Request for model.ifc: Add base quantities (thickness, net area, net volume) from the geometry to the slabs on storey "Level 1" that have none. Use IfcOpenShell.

First a look at what the model holds.

```python
import ifcopenshell
import ifcopenshell.util.element
import ifcopenshell.util.unit

model = ifcopenshell.open("model.ifc")
print(model.schema)
for unit_type in ("LENGTHUNIT", "AREAUNIT", "VOLUMEUNIT"):
    print(unit_type, ifcopenshell.util.unit.calculate_unit_scale(model, unit_type))
storey = next(s for s in model.by_type("IfcBuildingStorey") if s.Name == "Level 1")
slabs = [e for e in ifcopenshell.util.element.get_decomposition(storey) if e.is_a("IfcSlab")]
for e in sorted(slabs, key=lambda e: e.id()):
    print(e.id(), e.is_a(), e.Name, list(ifcopenshell.util.element.get_psets(e, qtos_only=True)), sep=" | ")
```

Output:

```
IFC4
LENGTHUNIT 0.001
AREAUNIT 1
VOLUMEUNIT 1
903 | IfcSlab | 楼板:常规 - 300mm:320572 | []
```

```python
import ifcopenshell
import ifcopenshell.api.pset
import ifcopenshell.geom
import ifcopenshell.util.element
import ifcopenshell.util.shape
import ifcopenshell.util.unit

model = ifcopenshell.open("model.ifc")
unit_scale = ifcopenshell.util.unit.calculate_unit_scale(model)
area_scale = ifcopenshell.util.unit.calculate_unit_scale(model, "AREAUNIT")
volume_scale = ifcopenshell.util.unit.calculate_unit_scale(model, "VOLUMEUNIT")
settings = ifcopenshell.geom.settings()

storey = next(s for s in model.by_type("IfcBuildingStorey") if s.Name == "Level 1")
slabs = [e for e in ifcopenshell.util.element.get_decomposition(storey) if e.is_a("IfcSlab")]

for e in sorted(slabs, key=lambda e: e.id()):
    if ifcopenshell.util.element.get_psets(e, qtos_only=True, should_inherit=False):
        continue
    # Geometry comes back in metres, in the element's own axes.
    shape = ifcopenshell.geom.create_shape(settings, e)
    values = {
        "Width": ifcopenshell.util.shape.get_z(shape.geometry) / unit_scale,
        "NetArea": ifcopenshell.util.shape.get_footprint_area(shape.geometry) / area_scale,
        "NetVolume": ifcopenshell.util.shape.get_volume(shape.geometry) / volume_scale,
    }
    qto = ifcopenshell.api.pset.add_qto(model, product=e, name="Qto_SlabBaseQuantities")
    ifcopenshell.api.pset.edit_qto(model, qto=qto, properties=values)
    print(e.id(), {k: round(v, 3) for k, v in values.items()})

model.write("model_edited.ifc")
```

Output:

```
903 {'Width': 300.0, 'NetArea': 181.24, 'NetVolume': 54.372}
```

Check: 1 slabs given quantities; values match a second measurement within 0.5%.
